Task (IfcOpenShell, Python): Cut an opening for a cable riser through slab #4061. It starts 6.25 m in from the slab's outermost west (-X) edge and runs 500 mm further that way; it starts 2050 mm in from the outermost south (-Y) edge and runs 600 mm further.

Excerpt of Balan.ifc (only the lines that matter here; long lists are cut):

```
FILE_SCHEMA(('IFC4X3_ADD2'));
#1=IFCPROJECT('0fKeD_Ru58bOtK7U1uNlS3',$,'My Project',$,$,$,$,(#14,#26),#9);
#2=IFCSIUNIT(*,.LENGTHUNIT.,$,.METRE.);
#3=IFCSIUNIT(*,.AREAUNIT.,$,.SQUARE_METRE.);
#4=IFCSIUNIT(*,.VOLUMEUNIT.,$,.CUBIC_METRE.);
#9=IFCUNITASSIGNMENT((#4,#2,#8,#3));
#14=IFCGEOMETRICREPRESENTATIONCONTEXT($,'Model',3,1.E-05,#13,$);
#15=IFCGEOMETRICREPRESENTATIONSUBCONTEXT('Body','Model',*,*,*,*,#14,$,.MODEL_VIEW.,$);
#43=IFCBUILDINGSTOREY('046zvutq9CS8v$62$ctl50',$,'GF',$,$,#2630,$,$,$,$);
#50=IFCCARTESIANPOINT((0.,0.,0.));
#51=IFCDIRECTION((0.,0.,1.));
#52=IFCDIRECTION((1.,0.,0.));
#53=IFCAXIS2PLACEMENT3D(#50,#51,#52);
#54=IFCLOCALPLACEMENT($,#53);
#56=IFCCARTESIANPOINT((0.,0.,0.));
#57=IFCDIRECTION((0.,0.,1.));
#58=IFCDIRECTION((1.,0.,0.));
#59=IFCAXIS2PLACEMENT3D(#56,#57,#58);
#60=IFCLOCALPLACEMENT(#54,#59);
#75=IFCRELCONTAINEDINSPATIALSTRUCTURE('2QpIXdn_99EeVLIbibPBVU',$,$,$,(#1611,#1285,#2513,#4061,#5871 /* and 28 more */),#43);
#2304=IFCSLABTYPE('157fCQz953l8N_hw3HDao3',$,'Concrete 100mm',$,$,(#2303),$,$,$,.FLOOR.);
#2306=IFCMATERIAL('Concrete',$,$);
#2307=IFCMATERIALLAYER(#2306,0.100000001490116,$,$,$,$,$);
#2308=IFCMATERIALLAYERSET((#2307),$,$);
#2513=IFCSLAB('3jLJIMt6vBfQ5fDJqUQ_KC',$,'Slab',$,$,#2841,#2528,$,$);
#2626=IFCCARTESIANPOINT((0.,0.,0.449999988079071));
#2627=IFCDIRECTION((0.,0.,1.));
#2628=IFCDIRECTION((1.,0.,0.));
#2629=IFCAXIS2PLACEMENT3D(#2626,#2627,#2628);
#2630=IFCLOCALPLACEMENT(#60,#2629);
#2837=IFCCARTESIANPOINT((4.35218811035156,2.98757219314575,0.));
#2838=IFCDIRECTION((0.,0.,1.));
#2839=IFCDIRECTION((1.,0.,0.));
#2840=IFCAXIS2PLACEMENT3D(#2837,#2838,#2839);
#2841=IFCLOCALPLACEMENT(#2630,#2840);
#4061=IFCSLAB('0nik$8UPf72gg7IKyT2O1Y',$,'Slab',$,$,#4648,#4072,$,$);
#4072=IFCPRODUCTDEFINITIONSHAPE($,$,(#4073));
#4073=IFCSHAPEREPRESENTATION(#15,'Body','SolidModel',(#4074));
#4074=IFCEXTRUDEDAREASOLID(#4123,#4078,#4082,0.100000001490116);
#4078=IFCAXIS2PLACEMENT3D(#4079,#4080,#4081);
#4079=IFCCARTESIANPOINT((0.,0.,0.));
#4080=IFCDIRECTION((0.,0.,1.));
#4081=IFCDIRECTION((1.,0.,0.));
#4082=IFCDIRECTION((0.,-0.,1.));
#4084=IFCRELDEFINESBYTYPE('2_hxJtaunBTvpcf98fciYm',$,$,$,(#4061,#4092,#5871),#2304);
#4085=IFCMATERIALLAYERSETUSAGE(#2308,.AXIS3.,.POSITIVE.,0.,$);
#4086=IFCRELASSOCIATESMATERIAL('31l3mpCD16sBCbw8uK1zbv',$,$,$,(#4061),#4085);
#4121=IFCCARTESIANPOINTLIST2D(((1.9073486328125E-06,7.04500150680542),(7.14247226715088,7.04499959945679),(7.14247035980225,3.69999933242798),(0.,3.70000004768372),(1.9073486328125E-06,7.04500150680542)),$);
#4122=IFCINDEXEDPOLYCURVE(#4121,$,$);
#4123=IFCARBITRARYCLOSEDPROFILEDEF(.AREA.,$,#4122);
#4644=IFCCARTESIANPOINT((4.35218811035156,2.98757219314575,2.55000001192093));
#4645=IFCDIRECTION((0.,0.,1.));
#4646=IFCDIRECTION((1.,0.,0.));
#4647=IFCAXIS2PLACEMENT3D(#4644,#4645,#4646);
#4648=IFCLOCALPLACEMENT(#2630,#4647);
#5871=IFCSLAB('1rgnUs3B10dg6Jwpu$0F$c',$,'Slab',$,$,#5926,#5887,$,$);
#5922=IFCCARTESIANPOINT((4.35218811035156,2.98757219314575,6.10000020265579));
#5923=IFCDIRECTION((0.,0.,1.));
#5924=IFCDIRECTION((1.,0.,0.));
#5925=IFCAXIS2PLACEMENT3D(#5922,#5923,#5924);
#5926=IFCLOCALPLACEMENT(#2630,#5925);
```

```python
import numpy as np
import ifcopenshell
import ifcopenshell.api.feature
import ifcopenshell.api.geometry
import ifcopenshell.api.root
import ifcopenshell.geom
import ifcopenshell.util.placement
import ifcopenshell.util.representation
import ifcopenshell.util.shape
import ifcopenshell.util.unit

model = ifcopenshell.open("Balan.ifc")
unit_scale = ifcopenshell.util.unit.calculate_unit_scale(model)
settings = ifcopenshell.geom.settings()


def volume(element):
    """Net volume in cubic metres, openings subtracted."""
    shape = ifcopenshell.geom.create_shape(settings, element)
    return ifcopenshell.util.shape.get_volume(shape.geometry)


slab = model.by_id(4061)
before = volume(slab)

# Extent in the slab's own axes, in metres. The edges named are its -X and -Y sides.
slab_shape = ifcopenshell.geom.create_shape(settings, slab)
vertices = ifcopenshell.util.shape.get_vertices(slab_shape.geometry)
x_min, y_min, bottom = vertices.min(axis=0)
top = vertices[:, 2].max()

opening = ifcopenshell.api.root.create_entity(model, ifc_class="IfcOpeningElement", name="Cable riser opening", predefined_type="OPENING")
context = ifcopenshell.util.representation.get_context(model, "Model", "Body", "MODEL_VIEW")
width, depth = 0.5, 0.6
outline = [(0.0, 0.0), (width, 0.0), (width, depth), (0.0, depth), (0.0, 0.0)]
# Overshoot both faces by 50 mm so the cut is clean.
shape = ifcopenshell.api.geometry.add_slab_representation(
    model, context=context, depth=top - bottom + 0.1, polyline=outline
)
ifcopenshell.api.geometry.assign_representation(model, product=opening, representation=shape)

matrix = ifcopenshell.util.placement.get_local_placement(slab.ObjectPlacement)
matrix[:, 3] = matrix @ np.append(np.array([x_min + 6.25, y_min + 2.05, bottom - 0.05]) / unit_scale, 1.0)
ifcopenshell.api.geometry.edit_object_placement(model, product=opening, matrix=matrix, is_si=False)
ifcopenshell.api.feature.add_feature(model, feature=opening, element=slab)

after = volume(slab)

print(f"slab volume {before:.3f} -> {after:.3f} m3")

model.write("Balan_rev.ifc")
```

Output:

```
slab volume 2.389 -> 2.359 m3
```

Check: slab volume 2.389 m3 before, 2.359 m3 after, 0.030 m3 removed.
